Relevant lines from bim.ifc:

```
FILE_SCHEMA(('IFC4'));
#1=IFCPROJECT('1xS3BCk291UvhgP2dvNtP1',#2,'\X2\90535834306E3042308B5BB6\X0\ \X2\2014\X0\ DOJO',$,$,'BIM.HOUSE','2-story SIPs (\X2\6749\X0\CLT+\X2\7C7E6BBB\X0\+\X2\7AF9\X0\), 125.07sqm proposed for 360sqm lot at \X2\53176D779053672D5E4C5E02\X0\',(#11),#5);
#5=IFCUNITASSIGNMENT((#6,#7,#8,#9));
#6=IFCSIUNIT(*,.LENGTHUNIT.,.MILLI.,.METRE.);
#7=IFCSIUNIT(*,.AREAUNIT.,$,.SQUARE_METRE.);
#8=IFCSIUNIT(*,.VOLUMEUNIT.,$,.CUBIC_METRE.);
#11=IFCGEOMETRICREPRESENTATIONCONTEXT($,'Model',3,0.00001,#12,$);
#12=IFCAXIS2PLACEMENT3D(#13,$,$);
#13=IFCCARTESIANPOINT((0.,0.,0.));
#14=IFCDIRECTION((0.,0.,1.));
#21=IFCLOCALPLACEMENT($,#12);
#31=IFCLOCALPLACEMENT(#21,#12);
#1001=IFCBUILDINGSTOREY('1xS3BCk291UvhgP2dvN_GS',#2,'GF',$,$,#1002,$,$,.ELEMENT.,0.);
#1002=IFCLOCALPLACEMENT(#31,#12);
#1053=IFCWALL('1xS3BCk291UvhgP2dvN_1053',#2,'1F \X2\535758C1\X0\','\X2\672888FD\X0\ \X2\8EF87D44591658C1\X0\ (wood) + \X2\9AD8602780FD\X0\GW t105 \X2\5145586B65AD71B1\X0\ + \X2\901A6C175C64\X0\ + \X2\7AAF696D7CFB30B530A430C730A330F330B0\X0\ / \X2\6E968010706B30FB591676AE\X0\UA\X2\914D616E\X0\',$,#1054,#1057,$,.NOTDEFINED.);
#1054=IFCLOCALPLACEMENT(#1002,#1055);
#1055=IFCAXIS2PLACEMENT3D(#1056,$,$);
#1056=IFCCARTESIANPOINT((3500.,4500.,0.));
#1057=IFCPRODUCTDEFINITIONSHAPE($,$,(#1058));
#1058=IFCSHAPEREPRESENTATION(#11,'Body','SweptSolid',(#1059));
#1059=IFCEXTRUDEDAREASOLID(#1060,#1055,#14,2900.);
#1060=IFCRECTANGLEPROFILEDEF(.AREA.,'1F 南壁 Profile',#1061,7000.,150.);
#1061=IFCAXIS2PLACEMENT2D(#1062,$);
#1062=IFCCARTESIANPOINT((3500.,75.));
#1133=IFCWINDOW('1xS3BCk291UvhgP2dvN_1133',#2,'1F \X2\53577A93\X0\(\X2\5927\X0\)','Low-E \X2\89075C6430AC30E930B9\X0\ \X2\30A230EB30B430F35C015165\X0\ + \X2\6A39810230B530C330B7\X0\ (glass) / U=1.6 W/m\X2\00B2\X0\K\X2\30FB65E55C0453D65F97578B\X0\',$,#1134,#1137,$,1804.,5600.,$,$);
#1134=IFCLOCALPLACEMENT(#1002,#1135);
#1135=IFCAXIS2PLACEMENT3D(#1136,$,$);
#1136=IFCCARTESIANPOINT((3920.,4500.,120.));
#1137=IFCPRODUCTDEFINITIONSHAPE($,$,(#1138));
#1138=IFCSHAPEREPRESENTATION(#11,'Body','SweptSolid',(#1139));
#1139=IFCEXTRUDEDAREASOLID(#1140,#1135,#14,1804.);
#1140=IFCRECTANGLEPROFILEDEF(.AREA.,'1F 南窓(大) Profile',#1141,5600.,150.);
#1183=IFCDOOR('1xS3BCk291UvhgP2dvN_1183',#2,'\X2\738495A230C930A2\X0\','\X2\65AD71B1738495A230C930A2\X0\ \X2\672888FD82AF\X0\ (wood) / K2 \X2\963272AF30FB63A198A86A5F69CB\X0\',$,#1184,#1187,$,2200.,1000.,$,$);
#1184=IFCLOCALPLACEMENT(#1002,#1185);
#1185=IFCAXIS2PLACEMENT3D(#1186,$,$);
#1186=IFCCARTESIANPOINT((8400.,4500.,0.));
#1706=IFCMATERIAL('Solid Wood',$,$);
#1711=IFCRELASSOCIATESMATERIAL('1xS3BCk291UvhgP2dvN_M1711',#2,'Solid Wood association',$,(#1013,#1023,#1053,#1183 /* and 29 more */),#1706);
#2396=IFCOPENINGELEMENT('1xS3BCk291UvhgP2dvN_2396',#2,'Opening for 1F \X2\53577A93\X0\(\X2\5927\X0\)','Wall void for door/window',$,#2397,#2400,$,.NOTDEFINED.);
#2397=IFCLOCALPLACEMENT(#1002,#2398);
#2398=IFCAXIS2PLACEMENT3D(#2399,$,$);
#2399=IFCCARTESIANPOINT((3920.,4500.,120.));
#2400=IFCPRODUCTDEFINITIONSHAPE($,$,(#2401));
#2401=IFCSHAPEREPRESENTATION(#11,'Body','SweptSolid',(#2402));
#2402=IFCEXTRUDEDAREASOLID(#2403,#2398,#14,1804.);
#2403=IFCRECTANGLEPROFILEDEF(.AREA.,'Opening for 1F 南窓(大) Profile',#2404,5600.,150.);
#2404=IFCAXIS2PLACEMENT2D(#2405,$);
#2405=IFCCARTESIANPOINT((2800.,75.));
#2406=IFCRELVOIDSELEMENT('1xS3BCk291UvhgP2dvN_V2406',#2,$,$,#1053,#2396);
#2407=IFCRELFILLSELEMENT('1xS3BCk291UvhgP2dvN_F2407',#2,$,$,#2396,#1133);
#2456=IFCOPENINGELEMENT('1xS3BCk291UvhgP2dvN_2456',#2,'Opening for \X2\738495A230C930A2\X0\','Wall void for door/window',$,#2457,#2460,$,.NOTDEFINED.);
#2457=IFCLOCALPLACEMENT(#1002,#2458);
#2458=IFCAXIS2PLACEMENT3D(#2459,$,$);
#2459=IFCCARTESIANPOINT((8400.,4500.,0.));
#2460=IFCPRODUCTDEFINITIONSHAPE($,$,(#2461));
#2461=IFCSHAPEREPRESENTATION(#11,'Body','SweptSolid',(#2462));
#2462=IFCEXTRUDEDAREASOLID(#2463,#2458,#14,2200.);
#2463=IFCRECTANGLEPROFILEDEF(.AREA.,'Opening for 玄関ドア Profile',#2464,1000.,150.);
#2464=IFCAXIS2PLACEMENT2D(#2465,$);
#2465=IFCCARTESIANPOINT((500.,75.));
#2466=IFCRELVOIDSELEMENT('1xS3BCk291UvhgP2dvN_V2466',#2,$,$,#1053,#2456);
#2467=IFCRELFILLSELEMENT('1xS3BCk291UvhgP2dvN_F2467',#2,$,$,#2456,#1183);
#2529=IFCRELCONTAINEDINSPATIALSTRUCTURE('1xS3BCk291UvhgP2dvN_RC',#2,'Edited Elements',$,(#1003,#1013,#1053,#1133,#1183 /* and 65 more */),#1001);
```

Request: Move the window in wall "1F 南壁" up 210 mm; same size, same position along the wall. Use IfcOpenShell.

```python
import numpy as np
import ifcopenshell
import ifcopenshell.api.geometry
import ifcopenshell.util.placement
import ifcopenshell.util.unit

model = ifcopenshell.open("bim.ifc")
unit_scale = ifcopenshell.util.unit.calculate_unit_scale(model)

window = model.by_guid("1xS3BCk291UvhgP2dvN_1133")
opening = window.FillsVoids[0].RelatingOpeningElement
dz = 210.0

shift = np.array([0.0, 0.0, dz])
# The window is not placed relative to its opening, so move both.
for product in (opening, window):
    matrix = ifcopenshell.util.placement.get_local_placement(product.ObjectPlacement)
    matrix[:3, 3] += shift
    ifcopenshell.api.geometry.edit_object_placement(model, product=product, matrix=matrix, is_si=False)

print(f"moved by {dz * unit_scale:+.3f} m")

model.write("bim-out.ifc")
```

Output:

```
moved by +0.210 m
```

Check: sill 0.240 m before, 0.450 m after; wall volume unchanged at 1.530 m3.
